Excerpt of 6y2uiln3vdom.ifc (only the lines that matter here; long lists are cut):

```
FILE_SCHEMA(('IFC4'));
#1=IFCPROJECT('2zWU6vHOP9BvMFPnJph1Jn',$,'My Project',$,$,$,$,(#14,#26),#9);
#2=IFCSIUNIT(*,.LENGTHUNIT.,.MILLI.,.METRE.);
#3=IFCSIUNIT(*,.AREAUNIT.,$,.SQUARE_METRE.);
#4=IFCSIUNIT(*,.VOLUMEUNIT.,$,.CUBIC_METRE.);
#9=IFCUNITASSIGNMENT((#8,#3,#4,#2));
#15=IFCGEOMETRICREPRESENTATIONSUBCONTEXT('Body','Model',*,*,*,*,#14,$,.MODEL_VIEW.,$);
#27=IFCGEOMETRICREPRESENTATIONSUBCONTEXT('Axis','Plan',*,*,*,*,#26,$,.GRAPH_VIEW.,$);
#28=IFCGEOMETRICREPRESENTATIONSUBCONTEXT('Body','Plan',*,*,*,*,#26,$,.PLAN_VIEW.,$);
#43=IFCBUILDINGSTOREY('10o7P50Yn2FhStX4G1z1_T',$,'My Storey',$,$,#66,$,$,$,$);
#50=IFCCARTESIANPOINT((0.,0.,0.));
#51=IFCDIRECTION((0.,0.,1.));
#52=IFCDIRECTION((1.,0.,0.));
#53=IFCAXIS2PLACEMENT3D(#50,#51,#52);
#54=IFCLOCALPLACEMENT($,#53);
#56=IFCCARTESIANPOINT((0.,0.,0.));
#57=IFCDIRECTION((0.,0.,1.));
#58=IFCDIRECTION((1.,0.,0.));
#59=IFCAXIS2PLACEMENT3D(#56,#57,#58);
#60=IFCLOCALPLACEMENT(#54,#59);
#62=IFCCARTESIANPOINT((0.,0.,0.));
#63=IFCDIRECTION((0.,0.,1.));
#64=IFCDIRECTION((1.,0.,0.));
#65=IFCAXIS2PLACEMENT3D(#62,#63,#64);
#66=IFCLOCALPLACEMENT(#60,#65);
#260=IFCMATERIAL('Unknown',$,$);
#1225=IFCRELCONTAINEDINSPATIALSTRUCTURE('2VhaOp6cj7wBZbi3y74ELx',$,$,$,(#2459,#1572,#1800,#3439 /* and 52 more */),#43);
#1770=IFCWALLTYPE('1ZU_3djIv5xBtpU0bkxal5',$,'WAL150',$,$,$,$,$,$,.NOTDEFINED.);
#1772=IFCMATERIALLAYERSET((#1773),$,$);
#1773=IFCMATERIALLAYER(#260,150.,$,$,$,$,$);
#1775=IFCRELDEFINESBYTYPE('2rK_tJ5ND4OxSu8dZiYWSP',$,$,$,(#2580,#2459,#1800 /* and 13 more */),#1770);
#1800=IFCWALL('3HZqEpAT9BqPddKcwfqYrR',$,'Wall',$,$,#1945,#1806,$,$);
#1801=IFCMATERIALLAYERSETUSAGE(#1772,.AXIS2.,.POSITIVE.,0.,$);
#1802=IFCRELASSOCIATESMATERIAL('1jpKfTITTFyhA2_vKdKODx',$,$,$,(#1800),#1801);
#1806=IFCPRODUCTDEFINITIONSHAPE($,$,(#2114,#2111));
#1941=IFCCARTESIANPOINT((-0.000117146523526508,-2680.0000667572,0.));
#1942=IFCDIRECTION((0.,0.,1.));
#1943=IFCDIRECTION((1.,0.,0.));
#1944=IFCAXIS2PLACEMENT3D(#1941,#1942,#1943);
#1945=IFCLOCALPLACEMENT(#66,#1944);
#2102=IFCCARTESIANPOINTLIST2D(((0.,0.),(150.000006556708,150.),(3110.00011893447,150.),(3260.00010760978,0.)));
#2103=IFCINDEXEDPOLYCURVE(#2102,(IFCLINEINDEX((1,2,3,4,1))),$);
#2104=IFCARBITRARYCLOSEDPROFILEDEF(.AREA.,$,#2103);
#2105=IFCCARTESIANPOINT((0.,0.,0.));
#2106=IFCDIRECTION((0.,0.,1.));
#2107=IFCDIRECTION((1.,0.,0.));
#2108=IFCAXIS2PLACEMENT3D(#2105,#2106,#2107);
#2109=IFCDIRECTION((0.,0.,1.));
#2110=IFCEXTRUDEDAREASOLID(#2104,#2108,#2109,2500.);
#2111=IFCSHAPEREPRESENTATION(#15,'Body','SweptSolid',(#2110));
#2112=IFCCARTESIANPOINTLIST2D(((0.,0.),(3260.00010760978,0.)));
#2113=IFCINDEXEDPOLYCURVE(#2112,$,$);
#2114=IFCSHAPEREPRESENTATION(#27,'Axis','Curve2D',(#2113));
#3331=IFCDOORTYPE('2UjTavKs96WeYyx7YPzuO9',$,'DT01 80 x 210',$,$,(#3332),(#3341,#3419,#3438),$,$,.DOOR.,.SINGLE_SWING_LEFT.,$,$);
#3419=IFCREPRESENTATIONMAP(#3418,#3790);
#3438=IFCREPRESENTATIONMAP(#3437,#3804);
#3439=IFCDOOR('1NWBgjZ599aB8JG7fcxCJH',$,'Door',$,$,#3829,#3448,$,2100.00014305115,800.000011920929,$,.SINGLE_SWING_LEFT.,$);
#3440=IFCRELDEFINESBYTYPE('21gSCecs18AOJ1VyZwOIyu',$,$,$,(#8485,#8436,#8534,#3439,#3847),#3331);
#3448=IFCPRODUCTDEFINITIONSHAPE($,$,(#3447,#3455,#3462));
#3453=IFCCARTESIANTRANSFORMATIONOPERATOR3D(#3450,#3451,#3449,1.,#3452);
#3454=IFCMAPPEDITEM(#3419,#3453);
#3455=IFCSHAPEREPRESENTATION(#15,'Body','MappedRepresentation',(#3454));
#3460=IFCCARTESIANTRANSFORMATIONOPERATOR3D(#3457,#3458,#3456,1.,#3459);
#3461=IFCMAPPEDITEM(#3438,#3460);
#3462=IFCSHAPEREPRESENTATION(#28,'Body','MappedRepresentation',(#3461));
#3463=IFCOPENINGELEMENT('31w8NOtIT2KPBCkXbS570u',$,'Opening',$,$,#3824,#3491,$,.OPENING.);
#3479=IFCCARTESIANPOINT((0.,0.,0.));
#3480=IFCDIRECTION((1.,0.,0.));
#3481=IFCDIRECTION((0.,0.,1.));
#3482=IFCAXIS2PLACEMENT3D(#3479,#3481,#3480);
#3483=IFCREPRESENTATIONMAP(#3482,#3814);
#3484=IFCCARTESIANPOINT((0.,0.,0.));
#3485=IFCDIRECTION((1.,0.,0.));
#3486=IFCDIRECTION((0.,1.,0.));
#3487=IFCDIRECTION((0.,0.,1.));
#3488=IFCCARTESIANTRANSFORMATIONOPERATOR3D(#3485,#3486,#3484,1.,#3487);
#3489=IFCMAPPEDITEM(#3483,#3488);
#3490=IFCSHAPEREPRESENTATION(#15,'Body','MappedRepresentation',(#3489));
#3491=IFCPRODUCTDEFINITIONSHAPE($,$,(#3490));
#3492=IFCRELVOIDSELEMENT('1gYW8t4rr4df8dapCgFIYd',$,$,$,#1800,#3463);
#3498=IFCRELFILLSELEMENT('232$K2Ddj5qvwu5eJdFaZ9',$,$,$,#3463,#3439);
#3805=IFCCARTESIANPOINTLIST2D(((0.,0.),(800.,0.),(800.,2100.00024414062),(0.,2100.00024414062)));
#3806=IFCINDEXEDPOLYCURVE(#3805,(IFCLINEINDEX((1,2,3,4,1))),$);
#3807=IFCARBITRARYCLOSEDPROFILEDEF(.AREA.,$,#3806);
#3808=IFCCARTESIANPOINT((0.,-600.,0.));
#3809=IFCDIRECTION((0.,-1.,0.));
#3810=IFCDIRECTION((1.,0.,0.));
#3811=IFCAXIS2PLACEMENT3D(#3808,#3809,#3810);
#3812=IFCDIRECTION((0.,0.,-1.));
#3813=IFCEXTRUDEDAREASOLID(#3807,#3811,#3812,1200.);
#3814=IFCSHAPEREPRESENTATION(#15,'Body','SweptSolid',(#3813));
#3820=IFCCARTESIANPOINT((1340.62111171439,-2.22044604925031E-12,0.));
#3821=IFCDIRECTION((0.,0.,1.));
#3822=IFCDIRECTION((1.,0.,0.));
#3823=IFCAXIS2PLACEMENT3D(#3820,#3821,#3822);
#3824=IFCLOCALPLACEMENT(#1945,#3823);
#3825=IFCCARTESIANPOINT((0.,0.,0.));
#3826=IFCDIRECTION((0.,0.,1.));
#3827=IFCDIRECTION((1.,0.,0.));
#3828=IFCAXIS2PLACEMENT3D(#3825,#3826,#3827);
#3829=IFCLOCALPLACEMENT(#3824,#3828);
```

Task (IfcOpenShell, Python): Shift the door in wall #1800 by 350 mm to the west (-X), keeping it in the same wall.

```python
import ifcopenshell
import ifcopenshell.api.geometry
import ifcopenshell.util.placement
import ifcopenshell.util.unit

model = ifcopenshell.open("6y2uiln3vdom.ifc")
unit_scale = ifcopenshell.util.unit.calculate_unit_scale(model)

door = model.by_guid("1NWBgjZ599aB8JG7fcxCJH")
opening = door.FillsVoids[0].RelatingOpeningElement
wall = opening.VoidsElements[0].RelatingBuildingElement

wall_matrix = ifcopenshell.util.placement.get_local_placement(wall.ObjectPlacement)
shift = wall_matrix[:3, 0] * -0.35 / unit_scale
before = ifcopenshell.util.placement.get_local_placement(door.ObjectPlacement)[:3, 3].copy()

# The door is placed relative to its opening, so it follows when the opening moves.
matrix = ifcopenshell.util.placement.get_local_placement(opening.ObjectPlacement)
matrix[:3, 3] += shift
ifcopenshell.api.geometry.edit_object_placement(
    model, product=opening, matrix=matrix, is_si=False, should_transform_children=True
)

after = ifcopenshell.util.placement.get_local_placement(door.ObjectPlacement)[:3, 3]
print("door moved by", (after - before).round(3) + 0.0)

model.write("6y2uiln3vdom_edited.ifc")
```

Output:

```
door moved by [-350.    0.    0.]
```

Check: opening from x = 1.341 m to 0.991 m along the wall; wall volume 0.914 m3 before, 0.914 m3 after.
